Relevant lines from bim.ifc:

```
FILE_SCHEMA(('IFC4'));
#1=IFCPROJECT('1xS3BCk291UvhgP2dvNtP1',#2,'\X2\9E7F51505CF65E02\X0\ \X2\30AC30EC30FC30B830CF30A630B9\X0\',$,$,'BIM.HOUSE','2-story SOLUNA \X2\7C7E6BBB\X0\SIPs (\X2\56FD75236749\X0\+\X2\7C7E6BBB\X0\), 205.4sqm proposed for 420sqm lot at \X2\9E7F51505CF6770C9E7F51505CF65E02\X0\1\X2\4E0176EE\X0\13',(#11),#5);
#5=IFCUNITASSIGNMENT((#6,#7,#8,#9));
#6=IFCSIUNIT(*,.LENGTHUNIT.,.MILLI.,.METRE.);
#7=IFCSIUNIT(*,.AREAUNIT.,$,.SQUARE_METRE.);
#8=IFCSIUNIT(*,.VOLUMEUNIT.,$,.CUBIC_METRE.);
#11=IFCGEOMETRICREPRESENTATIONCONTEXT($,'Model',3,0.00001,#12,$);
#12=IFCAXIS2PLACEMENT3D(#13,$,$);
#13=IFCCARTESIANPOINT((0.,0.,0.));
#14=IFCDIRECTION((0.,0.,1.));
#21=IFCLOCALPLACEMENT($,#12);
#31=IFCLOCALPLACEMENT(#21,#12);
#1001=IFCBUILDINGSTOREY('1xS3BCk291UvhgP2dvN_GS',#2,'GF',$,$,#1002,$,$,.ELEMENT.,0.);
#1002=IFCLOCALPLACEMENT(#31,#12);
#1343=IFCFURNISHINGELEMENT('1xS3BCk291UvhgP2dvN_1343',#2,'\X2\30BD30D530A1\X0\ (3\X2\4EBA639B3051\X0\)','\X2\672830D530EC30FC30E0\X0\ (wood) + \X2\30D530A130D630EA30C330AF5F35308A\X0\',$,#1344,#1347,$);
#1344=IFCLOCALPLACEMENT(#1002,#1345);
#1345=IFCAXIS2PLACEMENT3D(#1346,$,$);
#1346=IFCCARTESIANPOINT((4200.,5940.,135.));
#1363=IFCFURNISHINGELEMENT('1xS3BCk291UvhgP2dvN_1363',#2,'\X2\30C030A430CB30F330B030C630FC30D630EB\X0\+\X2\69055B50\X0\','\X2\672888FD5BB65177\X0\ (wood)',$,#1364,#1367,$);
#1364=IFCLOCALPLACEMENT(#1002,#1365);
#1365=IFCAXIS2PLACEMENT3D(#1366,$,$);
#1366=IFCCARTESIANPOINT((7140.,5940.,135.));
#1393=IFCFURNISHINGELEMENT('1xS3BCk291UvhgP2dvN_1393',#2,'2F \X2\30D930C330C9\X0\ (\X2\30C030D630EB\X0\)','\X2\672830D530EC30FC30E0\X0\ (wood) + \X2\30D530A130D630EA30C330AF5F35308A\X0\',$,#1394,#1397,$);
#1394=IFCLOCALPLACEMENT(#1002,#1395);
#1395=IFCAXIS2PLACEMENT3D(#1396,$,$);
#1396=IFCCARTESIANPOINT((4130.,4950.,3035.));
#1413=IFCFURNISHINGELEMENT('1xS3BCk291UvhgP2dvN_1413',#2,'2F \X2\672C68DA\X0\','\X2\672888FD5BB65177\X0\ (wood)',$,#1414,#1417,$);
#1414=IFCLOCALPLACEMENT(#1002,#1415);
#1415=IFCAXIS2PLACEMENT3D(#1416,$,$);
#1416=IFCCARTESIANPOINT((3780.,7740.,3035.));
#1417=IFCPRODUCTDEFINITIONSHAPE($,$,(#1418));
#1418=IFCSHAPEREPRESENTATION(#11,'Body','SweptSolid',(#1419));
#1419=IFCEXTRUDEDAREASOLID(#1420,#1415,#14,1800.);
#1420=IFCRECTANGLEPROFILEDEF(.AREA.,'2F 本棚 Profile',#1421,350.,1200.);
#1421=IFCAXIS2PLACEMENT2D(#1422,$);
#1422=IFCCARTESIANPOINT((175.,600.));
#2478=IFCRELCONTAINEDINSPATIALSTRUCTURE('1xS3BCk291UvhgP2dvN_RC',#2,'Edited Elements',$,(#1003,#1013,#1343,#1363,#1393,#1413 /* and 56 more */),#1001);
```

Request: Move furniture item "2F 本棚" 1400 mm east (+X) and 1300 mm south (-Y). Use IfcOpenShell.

```python
import ifcopenshell
import ifcopenshell.api.geometry
import ifcopenshell.util.placement
import ifcopenshell.util.unit

model = ifcopenshell.open("bim.ifc")
unit_scale = ifcopenshell.util.unit.calculate_unit_scale(model)

item = model.by_guid("1xS3BCk291UvhgP2dvN_1413")
matrix = ifcopenshell.util.placement.get_local_placement(item.ObjectPlacement)
matrix[0, 3] += 1.4 / unit_scale
matrix[1, 3] -= 1.3 / unit_scale
ifcopenshell.api.geometry.edit_object_placement(model, product=item, matrix=matrix, is_si=False)

print(ifcopenshell.util.placement.get_local_placement(item.ObjectPlacement).round(3) + 0.0)

model.write("bim_edited.ifc")
```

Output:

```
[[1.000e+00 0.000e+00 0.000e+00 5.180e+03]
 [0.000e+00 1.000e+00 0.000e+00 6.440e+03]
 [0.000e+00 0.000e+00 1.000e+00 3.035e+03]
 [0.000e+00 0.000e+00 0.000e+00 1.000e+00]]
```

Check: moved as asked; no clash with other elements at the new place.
